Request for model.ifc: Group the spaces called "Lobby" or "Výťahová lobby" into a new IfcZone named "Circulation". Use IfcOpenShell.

First a look at what the model holds.

```python
import ifcopenshell

model = ifcopenshell.open("model.ifc")
print(model.schema)
seen = {}
for space in model.by_type("IfcSpace"):
    seen[space.LongName] = seen.get(space.LongName, 0) + 1
for name, count in sorted(seen.items(), key=str):
    print(count, "x", name)
print("zones:", [z.Name for z in model.by_type("IfcZone")][:20])
```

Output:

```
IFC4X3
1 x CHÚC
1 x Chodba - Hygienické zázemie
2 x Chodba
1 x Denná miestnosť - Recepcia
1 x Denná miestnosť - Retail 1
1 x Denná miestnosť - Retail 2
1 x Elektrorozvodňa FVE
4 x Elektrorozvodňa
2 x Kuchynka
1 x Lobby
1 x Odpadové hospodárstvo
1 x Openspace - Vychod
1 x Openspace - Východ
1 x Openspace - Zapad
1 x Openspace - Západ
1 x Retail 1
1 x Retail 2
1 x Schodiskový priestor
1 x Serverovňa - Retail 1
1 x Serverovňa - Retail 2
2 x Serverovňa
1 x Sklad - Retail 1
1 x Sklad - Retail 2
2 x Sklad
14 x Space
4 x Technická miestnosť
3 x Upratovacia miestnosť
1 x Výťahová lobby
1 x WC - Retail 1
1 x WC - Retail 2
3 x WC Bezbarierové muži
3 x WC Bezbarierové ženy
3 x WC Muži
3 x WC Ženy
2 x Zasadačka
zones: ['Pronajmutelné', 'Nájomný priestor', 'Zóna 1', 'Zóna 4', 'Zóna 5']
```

```python
import ifcopenshell
import ifcopenshell.api.group
import ifcopenshell.api.root

model = ifcopenshell.open("model.ifc")

names = {"Lobby", "Výťahová lobby"}
spaces = [s for s in model.by_type("IfcSpace") if s.LongName in names]

zone = ifcopenshell.api.root.create_entity(model, ifc_class="IfcZone", name="Circulation")
ifcopenshell.api.group.assign_group(model, products=spaces, group=zone)
print(len(spaces), "spaces in", zone.Name)

model.write("model_updated.ifc")
```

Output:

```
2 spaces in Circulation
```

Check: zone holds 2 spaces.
